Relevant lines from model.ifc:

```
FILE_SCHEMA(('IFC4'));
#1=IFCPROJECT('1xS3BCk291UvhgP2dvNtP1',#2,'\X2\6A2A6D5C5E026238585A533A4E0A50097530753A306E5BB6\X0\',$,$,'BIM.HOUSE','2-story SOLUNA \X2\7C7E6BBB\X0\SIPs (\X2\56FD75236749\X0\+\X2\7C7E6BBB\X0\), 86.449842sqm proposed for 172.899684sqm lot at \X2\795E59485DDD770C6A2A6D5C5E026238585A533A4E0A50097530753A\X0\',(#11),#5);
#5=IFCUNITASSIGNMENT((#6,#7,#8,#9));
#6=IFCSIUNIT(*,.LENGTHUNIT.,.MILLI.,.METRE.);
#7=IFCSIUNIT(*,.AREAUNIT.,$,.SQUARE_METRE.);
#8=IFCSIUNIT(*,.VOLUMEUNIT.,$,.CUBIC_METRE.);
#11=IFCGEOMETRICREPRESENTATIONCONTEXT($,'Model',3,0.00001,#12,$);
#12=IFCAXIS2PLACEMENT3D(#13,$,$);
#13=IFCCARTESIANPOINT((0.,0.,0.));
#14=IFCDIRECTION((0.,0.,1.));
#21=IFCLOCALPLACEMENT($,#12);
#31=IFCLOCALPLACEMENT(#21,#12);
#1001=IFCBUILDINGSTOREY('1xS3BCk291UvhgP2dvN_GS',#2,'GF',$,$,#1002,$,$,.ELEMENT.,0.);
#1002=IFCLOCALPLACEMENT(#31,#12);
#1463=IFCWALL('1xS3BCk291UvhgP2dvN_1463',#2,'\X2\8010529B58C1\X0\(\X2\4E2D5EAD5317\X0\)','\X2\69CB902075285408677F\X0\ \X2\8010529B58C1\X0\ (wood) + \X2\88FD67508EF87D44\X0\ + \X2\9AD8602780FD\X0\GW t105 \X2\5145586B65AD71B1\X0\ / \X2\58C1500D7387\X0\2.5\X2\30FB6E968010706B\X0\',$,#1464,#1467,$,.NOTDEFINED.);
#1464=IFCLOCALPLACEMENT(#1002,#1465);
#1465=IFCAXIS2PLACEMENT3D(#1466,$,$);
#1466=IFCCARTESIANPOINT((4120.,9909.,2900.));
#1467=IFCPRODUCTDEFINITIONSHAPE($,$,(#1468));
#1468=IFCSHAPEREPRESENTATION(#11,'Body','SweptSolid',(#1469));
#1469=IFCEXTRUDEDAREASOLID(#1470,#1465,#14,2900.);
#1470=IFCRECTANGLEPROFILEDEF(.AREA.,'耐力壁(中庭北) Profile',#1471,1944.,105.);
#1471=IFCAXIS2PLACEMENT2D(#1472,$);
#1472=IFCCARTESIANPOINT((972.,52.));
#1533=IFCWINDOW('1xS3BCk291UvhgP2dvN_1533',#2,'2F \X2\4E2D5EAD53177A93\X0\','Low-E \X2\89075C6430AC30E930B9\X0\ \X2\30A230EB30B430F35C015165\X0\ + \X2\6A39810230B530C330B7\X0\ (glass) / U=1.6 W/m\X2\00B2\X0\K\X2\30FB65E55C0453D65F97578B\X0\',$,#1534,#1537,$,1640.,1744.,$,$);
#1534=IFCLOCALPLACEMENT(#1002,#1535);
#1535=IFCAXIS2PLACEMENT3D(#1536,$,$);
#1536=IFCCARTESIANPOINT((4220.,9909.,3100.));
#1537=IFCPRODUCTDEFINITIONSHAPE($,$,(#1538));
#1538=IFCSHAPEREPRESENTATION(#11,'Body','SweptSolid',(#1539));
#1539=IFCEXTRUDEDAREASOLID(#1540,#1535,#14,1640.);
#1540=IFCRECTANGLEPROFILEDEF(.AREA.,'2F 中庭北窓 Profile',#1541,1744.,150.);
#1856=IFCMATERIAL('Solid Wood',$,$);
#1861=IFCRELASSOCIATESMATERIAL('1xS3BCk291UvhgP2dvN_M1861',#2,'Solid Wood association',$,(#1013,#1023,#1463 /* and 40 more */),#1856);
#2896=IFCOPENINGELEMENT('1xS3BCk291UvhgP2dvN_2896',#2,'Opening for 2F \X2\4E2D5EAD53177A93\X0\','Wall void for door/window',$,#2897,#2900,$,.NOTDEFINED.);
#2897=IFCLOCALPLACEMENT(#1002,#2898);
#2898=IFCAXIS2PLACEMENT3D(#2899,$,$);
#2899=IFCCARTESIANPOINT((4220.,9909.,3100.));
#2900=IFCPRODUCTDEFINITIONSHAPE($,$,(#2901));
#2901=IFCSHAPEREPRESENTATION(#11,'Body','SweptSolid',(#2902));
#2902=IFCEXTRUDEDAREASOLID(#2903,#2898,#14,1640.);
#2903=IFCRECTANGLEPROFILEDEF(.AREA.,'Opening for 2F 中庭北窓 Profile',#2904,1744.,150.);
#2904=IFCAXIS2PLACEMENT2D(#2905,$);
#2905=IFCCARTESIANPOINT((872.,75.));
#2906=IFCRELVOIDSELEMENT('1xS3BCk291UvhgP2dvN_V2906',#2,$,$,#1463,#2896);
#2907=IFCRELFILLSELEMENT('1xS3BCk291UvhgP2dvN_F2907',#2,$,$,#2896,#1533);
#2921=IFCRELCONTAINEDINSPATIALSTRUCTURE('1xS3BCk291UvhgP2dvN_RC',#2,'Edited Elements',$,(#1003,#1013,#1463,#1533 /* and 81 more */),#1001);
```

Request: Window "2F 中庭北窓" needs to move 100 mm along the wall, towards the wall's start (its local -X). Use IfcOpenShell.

```python
import ifcopenshell
import ifcopenshell.api.geometry
import ifcopenshell.util.placement

model = ifcopenshell.open("model.ifc")

window = model.by_id(1533)
opening = window.FillsVoids[0].RelatingOpeningElement
wall = opening.VoidsElements[0].RelatingBuildingElement

wall_matrix = ifcopenshell.util.placement.get_local_placement(wall.ObjectPlacement)
shift = wall_matrix[:3, 0] * -100.0
before = ifcopenshell.util.placement.get_local_placement(window.ObjectPlacement)[:3, 3].copy()

# The window is not placed relative to its opening, so move both.
for product in (opening, window):
    matrix = ifcopenshell.util.placement.get_local_placement(product.ObjectPlacement)
    matrix[:3, 3] += shift
    ifcopenshell.api.geometry.edit_object_placement(model, product=product, matrix=matrix, is_si=False)

after = ifcopenshell.util.placement.get_local_placement(window.ObjectPlacement)[:3, 3]
print("window moved by", (after - before).round(3) + 0.0)

model.write("model_rev.ifc")
```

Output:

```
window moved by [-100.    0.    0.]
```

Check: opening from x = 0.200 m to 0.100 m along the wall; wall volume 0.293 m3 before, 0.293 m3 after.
